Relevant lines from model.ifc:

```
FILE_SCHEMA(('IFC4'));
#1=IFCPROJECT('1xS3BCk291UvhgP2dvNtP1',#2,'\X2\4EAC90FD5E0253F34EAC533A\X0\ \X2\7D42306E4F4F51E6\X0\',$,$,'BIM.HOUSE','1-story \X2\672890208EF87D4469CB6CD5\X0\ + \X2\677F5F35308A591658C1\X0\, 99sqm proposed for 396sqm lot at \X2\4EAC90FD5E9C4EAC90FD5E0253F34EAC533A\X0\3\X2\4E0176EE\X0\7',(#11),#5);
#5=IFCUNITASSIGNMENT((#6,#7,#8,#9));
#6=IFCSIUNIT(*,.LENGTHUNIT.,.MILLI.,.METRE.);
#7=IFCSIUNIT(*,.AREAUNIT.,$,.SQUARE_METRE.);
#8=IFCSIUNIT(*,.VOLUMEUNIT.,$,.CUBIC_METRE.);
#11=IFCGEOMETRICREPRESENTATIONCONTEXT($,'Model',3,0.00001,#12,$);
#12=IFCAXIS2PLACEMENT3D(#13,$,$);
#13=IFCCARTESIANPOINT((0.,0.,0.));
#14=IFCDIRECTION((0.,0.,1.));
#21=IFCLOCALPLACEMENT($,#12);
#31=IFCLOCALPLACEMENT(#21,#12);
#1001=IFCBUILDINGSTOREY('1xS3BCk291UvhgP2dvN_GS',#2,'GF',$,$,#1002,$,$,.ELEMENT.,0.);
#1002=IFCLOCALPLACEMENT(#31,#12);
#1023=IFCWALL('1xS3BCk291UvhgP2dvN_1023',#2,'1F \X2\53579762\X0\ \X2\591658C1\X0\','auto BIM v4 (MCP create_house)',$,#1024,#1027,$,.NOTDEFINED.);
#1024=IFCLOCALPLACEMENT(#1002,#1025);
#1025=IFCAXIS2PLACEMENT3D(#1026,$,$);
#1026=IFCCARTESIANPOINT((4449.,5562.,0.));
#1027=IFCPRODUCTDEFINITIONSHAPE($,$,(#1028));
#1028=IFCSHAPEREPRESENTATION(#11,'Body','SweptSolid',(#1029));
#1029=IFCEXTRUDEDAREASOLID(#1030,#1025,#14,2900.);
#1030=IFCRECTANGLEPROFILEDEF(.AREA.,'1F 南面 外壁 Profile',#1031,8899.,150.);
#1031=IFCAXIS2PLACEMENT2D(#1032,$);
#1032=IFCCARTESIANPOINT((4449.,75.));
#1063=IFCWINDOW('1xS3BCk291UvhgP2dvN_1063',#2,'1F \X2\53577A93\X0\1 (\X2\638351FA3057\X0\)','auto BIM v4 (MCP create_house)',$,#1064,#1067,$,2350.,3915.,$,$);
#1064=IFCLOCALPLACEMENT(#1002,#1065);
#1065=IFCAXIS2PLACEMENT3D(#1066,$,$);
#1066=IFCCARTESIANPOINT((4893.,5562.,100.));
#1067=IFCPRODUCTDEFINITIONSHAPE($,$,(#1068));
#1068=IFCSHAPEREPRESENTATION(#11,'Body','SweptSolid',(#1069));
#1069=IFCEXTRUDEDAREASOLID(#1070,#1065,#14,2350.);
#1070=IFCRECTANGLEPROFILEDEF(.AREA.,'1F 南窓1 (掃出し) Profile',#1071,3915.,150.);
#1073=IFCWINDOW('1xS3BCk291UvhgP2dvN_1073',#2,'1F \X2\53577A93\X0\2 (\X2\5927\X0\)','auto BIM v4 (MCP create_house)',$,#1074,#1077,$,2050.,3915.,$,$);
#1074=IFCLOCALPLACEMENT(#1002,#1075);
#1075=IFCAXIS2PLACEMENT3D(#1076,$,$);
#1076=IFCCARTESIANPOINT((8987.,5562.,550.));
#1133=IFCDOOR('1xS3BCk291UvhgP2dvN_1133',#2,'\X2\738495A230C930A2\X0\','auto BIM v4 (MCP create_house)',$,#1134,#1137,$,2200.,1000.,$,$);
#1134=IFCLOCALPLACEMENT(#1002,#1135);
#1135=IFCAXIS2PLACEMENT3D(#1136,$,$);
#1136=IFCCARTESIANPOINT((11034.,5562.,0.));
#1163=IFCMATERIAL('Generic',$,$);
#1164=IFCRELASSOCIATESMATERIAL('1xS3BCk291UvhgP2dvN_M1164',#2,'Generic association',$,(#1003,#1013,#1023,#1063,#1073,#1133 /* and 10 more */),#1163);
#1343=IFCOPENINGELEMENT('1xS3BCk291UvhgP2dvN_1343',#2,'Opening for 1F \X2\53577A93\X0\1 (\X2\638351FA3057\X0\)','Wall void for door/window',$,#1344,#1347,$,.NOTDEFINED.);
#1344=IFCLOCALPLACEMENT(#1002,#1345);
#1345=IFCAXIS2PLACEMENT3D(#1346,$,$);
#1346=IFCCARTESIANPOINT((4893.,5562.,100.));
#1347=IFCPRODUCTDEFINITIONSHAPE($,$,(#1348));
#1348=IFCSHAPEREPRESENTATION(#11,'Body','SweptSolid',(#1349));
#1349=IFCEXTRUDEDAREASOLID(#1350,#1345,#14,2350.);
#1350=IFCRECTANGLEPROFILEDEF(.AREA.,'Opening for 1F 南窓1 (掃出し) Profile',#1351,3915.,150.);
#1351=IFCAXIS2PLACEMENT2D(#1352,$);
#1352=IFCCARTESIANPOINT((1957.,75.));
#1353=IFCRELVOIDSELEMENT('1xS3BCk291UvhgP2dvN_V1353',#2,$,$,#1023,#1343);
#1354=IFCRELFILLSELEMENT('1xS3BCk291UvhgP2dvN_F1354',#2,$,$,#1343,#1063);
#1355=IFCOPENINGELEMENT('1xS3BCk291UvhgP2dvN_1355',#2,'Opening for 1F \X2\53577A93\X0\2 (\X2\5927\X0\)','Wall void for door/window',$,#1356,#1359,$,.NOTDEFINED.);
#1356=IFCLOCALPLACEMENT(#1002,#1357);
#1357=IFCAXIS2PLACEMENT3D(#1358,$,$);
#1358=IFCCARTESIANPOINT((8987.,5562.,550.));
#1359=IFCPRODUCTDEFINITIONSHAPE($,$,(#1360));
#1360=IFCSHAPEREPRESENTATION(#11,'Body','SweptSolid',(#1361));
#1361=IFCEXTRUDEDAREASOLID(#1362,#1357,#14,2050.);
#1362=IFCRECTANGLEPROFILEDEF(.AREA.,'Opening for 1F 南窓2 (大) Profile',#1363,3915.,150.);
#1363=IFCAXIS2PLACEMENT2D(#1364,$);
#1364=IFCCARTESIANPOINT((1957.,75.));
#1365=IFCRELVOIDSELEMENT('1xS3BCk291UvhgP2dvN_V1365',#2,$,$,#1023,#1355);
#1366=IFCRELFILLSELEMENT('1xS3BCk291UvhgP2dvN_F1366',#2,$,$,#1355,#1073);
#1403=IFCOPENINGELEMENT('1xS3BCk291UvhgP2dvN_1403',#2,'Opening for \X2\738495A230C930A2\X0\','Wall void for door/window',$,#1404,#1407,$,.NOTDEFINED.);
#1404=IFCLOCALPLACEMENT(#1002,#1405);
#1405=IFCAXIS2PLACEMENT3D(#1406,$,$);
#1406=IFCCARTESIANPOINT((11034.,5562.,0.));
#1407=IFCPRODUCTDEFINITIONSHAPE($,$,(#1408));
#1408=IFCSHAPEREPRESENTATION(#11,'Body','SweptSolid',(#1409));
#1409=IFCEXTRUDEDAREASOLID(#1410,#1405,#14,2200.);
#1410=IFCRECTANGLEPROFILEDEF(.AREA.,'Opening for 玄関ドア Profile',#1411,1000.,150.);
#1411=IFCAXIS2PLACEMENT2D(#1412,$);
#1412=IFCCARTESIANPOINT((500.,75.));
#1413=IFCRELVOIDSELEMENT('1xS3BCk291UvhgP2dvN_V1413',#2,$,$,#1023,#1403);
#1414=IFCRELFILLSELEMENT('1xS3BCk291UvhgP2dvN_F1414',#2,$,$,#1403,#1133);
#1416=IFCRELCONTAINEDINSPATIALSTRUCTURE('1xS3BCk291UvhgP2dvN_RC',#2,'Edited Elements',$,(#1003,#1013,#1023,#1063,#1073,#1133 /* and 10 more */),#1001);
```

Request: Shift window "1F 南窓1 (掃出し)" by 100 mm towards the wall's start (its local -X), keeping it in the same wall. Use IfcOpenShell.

```python
import ifcopenshell
import ifcopenshell.api.geometry
import ifcopenshell.util.placement
import ifcopenshell.util.unit

model = ifcopenshell.open("model.ifc")
unit_scale = ifcopenshell.util.unit.calculate_unit_scale(model)

window = model.by_id(1063)
opening = window.FillsVoids[0].RelatingOpeningElement
wall = opening.VoidsElements[0].RelatingBuildingElement

wall_matrix = ifcopenshell.util.placement.get_local_placement(wall.ObjectPlacement)
shift = wall_matrix[:3, 0] * -0.1 / unit_scale
before = ifcopenshell.util.placement.get_local_placement(window.ObjectPlacement)[:3, 3].copy()

# The window is not placed relative to its opening, so move both.
for product in (opening, window):
    matrix = ifcopenshell.util.placement.get_local_placement(product.ObjectPlacement)
    matrix[:3, 3] += shift
    ifcopenshell.api.geometry.edit_object_placement(model, product=product, matrix=matrix, is_si=False)

after = ifcopenshell.util.placement.get_local_placement(window.ObjectPlacement)[:3, 3]
print("window moved by", (after - before).round(3) + 0.0)

model.write("model_v2.ifc")
```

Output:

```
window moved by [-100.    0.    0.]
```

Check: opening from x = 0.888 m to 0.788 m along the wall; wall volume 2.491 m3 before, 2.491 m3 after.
